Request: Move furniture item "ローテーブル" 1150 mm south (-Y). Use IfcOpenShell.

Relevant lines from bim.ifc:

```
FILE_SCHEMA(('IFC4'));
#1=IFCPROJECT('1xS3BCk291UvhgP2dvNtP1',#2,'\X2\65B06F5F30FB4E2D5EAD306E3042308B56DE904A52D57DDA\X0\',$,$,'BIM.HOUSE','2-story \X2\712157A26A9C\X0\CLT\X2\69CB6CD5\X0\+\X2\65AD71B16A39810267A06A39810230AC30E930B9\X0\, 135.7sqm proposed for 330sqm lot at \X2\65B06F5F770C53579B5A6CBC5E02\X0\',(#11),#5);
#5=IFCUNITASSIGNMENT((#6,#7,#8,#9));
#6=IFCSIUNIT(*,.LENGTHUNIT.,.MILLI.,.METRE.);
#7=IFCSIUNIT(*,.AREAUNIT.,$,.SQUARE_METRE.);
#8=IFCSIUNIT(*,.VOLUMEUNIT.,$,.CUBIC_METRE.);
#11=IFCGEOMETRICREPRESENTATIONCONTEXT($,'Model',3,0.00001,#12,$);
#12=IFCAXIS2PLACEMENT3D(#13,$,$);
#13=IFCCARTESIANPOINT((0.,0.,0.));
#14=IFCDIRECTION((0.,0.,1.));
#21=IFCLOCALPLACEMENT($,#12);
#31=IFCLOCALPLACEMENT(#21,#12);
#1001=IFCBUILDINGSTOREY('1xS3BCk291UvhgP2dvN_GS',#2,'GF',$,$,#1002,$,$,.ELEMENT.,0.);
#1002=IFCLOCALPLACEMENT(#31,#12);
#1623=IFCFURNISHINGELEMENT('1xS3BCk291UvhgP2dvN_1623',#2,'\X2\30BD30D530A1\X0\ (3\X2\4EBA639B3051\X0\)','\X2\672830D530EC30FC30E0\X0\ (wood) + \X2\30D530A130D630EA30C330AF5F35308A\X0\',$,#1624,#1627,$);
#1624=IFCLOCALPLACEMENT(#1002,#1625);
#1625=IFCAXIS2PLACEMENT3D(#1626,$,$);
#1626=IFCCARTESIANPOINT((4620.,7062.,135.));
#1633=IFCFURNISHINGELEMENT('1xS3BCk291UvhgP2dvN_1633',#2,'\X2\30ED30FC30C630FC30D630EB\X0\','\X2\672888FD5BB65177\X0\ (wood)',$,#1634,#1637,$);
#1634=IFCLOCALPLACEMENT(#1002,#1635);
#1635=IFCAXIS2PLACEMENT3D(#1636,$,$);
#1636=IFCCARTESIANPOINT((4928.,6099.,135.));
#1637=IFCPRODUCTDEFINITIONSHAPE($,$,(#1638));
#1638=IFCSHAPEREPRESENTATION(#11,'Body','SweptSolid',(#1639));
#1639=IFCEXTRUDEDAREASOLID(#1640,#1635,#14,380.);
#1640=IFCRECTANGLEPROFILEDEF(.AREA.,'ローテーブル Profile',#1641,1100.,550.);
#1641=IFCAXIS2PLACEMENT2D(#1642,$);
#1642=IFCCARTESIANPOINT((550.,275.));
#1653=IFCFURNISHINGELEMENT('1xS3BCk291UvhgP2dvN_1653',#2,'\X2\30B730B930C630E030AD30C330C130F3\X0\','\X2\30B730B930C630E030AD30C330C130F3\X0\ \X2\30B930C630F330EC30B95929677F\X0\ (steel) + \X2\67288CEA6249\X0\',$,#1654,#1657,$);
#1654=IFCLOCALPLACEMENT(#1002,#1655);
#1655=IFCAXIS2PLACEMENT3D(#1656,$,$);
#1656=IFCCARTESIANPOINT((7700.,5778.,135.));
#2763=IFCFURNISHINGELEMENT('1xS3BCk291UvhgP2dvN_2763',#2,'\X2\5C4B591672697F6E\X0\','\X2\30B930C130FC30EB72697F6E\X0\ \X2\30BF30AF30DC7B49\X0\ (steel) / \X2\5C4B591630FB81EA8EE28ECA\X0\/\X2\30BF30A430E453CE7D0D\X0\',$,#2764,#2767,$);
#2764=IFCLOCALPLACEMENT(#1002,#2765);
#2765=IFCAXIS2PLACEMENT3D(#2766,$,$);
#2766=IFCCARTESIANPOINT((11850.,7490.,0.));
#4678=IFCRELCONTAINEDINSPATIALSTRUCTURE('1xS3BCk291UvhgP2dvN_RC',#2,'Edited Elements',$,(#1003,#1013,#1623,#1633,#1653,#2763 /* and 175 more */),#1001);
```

```python
import ifcopenshell
import ifcopenshell.api.geometry
import ifcopenshell.util.placement
import ifcopenshell.util.unit

model = ifcopenshell.open("bim.ifc")
unit_scale = ifcopenshell.util.unit.calculate_unit_scale(model)

item = model.by_guid("1xS3BCk291UvhgP2dvN_1633")
matrix = ifcopenshell.util.placement.get_local_placement(item.ObjectPlacement)
matrix[1, 3] -= 1.15 / unit_scale
ifcopenshell.api.geometry.edit_object_placement(model, product=item, matrix=matrix, is_si=False)

print(ifcopenshell.util.placement.get_local_placement(item.ObjectPlacement).round(3) + 0.0)

model.write("bim_v2.ifc")
```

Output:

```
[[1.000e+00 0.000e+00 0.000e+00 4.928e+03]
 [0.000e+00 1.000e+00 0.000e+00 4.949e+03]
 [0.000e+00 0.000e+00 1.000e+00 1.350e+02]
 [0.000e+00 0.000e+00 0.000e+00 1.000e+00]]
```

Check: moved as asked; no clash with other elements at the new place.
